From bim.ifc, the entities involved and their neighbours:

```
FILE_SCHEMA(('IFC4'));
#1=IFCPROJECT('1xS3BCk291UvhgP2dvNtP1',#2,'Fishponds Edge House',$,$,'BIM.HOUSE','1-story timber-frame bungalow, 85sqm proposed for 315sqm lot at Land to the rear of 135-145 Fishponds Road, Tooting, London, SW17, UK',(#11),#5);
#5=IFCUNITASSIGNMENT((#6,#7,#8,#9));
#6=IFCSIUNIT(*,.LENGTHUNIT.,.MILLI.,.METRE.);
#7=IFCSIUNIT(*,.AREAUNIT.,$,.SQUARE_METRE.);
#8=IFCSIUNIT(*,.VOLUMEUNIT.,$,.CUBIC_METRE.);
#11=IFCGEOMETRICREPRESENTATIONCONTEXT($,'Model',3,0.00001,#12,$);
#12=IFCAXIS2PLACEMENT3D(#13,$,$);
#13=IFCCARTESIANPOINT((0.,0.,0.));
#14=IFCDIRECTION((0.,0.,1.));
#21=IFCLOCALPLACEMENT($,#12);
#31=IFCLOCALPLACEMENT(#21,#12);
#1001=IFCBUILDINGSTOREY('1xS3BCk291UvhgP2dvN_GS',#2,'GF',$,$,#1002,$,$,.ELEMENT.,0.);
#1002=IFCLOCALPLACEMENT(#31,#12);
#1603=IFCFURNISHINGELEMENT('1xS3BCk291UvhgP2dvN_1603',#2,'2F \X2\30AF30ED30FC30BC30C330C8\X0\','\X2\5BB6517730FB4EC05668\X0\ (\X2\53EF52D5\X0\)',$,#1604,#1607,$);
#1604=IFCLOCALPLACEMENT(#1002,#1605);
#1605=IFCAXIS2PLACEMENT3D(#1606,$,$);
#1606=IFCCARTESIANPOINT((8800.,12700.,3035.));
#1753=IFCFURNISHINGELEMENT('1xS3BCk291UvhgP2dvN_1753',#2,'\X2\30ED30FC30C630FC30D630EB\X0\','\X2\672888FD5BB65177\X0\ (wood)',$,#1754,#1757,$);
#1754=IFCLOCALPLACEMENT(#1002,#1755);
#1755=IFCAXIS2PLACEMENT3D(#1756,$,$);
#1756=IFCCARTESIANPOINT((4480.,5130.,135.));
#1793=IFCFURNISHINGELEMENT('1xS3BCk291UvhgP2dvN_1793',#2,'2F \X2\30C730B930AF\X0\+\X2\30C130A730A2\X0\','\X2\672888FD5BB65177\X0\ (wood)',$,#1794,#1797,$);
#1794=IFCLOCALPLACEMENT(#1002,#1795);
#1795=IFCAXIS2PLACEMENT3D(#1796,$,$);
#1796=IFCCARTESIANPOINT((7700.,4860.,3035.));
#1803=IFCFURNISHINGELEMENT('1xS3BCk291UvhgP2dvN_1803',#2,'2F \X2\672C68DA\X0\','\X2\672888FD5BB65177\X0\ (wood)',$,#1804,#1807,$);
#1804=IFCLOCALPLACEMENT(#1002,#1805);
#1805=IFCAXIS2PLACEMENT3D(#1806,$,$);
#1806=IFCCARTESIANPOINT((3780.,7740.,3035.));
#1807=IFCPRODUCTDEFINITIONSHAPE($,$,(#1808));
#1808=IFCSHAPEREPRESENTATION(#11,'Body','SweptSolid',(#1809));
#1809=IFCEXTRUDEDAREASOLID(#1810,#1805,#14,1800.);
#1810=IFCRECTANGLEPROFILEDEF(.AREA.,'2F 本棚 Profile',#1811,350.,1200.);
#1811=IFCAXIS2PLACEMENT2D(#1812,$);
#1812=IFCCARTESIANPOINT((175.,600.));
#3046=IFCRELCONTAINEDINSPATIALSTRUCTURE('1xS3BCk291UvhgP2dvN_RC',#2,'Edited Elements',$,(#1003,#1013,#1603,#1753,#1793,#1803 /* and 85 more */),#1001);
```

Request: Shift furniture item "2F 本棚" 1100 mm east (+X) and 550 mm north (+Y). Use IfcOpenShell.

```python
import ifcopenshell
import ifcopenshell.api.geometry
import ifcopenshell.util.placement
import ifcopenshell.util.unit

model = ifcopenshell.open("bim.ifc")
unit_scale = ifcopenshell.util.unit.calculate_unit_scale(model)

item = model.by_id(1803)
matrix = ifcopenshell.util.placement.get_local_placement(item.ObjectPlacement)
matrix[0, 3] += 1.1 / unit_scale
matrix[1, 3] += 0.55 / unit_scale
ifcopenshell.api.geometry.edit_object_placement(model, product=item, matrix=matrix, is_si=False)

print(ifcopenshell.util.placement.get_local_placement(item.ObjectPlacement).round(3) + 0.0)

model.write("bim_rev.ifc")
```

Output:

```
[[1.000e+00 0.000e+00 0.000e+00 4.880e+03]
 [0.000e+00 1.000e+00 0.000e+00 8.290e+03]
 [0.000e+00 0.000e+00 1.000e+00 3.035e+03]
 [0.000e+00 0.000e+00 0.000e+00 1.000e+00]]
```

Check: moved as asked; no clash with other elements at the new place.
